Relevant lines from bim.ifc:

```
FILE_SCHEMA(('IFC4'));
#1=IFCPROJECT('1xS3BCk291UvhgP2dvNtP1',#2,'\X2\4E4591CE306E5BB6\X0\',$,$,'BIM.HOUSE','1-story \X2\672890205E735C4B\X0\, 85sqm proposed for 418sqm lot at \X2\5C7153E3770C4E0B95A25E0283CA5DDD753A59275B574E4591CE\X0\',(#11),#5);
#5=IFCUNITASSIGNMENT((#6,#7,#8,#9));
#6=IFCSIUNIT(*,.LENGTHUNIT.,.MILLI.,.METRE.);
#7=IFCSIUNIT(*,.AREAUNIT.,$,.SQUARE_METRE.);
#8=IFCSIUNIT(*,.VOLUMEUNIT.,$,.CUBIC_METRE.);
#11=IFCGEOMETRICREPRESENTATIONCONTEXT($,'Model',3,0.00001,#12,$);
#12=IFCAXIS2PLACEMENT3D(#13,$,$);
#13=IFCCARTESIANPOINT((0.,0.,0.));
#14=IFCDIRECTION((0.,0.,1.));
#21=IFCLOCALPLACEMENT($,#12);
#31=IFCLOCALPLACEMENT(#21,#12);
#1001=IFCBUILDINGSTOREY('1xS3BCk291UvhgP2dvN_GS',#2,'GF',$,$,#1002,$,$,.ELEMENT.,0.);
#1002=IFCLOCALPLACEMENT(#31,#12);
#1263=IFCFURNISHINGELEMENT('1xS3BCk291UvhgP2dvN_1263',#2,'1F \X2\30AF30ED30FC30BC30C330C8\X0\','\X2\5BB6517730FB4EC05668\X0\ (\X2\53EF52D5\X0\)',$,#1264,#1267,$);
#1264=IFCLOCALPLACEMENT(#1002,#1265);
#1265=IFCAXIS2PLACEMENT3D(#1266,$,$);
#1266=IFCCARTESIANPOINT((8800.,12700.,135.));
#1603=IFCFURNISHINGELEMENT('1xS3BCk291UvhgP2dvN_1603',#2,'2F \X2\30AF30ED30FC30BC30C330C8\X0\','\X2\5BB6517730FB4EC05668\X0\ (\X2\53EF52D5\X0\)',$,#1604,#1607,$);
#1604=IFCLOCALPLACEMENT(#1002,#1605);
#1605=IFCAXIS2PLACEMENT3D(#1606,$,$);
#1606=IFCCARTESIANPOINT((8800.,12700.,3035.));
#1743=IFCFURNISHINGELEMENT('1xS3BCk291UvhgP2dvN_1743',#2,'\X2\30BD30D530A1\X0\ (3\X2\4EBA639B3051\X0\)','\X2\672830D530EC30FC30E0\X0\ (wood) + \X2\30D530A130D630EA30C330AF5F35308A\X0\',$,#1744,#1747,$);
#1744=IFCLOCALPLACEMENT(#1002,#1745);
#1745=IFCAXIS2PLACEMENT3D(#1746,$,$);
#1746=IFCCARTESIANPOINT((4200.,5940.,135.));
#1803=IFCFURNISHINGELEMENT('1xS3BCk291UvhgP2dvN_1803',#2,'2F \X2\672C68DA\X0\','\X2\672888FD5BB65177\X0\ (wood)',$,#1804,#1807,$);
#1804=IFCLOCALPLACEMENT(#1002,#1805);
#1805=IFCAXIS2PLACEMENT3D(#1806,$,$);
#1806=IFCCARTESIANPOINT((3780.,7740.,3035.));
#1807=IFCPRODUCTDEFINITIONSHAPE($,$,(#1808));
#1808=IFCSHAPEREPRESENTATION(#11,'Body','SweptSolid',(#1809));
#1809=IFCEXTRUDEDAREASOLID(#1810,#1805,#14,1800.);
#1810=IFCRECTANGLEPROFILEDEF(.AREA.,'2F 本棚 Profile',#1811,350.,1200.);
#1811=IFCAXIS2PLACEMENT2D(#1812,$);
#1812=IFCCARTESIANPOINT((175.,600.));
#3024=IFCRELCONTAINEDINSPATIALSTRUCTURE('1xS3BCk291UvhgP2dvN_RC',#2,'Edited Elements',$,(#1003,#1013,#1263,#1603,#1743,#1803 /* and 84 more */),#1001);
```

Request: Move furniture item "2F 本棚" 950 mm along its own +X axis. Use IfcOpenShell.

```python
import ifcopenshell
import ifcopenshell.api.geometry
import ifcopenshell.util.placement

model = ifcopenshell.open("bim.ifc")

item = model.by_guid("1xS3BCk291UvhgP2dvN_1803")
matrix = ifcopenshell.util.placement.get_local_placement(item.ObjectPlacement)
matrix[:3, 3] += matrix[:3, 0] * 950.0
ifcopenshell.api.geometry.edit_object_placement(model, product=item, matrix=matrix, is_si=False)

print(ifcopenshell.util.placement.get_local_placement(item.ObjectPlacement).round(3) + 0.0)

model.write("bim_v2.ifc")
```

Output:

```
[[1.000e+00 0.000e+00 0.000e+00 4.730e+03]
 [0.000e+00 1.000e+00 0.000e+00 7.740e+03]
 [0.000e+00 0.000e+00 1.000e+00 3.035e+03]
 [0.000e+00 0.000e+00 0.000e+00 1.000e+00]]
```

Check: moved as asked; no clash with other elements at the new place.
